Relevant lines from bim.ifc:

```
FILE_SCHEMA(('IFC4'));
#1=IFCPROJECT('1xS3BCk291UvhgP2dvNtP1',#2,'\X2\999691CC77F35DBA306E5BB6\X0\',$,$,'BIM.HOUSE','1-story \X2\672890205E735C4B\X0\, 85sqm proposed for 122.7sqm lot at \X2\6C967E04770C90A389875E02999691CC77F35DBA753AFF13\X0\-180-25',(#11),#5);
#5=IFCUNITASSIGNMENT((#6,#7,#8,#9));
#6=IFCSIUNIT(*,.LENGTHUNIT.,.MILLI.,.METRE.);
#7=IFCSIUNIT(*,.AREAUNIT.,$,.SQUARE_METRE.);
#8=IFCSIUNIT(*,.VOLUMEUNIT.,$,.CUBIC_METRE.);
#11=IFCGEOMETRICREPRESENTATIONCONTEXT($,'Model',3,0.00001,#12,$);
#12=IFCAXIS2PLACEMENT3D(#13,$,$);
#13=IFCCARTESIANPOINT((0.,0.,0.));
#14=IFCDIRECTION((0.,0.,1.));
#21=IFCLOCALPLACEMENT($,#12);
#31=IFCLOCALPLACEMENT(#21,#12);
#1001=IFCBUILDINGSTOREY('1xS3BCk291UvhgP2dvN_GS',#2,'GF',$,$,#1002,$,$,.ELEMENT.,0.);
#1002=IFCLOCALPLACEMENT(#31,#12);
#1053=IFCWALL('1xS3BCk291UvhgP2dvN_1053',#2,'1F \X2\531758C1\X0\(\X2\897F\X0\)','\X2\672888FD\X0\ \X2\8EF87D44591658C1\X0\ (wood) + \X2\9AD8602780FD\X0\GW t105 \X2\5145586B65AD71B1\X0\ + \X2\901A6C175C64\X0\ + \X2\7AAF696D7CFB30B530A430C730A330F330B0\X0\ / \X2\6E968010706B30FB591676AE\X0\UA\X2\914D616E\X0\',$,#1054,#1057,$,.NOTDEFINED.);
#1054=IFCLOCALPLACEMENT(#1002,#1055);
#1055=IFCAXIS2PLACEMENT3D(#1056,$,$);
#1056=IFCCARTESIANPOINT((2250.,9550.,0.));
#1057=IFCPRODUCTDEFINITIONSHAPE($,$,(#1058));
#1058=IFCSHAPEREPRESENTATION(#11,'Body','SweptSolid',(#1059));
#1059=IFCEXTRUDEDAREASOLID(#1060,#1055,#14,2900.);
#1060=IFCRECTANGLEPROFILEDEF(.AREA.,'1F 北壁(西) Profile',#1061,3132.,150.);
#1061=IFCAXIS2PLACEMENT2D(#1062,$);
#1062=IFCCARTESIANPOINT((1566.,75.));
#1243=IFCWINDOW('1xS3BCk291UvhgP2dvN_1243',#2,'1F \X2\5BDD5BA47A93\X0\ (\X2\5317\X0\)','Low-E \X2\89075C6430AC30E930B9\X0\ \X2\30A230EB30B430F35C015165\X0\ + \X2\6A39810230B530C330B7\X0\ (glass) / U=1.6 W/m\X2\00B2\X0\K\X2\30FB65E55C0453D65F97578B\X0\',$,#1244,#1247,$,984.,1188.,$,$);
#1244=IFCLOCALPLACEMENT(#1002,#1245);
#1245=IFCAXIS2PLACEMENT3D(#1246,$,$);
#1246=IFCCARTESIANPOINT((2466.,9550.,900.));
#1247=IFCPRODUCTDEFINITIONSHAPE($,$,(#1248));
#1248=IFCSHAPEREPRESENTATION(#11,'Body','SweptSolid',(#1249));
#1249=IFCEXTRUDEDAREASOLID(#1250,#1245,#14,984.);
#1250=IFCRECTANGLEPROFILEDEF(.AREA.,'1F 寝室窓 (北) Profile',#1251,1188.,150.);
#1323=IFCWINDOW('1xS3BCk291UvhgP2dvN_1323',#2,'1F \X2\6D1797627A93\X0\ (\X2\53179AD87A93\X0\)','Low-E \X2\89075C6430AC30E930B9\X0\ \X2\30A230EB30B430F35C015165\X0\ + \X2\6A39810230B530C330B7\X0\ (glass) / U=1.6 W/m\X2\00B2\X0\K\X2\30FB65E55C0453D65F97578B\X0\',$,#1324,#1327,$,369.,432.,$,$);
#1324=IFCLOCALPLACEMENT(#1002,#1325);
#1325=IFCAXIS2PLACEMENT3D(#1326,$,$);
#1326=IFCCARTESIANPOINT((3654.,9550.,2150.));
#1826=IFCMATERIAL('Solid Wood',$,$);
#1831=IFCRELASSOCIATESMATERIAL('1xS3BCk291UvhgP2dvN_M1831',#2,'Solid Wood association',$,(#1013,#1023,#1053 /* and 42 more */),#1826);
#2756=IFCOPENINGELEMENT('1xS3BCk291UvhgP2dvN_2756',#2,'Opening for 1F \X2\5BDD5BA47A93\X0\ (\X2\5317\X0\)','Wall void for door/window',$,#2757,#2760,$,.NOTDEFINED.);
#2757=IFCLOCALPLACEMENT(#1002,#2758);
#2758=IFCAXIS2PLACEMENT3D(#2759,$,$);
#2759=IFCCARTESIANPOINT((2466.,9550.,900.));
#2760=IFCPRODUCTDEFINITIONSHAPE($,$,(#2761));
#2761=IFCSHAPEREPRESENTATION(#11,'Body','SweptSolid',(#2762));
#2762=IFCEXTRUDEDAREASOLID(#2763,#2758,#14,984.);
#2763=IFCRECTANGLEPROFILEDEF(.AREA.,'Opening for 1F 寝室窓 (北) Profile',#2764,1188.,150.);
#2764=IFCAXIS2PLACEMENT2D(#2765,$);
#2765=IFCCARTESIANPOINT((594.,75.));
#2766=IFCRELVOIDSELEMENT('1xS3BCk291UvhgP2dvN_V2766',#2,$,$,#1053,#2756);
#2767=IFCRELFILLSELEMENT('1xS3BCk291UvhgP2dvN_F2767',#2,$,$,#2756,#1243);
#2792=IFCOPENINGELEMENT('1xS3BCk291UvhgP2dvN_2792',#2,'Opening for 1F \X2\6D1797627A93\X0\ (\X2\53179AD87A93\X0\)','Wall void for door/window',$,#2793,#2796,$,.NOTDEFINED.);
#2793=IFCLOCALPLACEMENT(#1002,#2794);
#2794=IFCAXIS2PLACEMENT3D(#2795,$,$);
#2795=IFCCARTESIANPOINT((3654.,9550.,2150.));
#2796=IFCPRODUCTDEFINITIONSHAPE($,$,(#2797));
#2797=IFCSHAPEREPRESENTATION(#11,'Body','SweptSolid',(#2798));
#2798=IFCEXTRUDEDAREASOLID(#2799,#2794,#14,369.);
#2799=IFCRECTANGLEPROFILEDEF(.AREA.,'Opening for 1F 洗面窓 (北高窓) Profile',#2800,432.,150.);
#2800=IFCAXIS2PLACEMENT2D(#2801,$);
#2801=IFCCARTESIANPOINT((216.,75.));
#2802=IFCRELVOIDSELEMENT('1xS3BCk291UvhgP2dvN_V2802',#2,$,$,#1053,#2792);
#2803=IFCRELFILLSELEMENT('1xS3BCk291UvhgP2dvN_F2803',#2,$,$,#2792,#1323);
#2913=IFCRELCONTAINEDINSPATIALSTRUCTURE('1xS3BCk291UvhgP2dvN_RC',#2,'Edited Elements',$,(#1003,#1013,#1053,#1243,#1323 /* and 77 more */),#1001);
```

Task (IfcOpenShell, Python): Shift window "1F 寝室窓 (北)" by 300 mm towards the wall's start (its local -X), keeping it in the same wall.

```python
import ifcopenshell
import ifcopenshell.api.geometry
import ifcopenshell.util.placement

model = ifcopenshell.open("bim.ifc")

window = model.by_guid("1xS3BCk291UvhgP2dvN_1243")
opening = window.FillsVoids[0].RelatingOpeningElement
wall = opening.VoidsElements[0].RelatingBuildingElement

wall_matrix = ifcopenshell.util.placement.get_local_placement(wall.ObjectPlacement)
shift = wall_matrix[:3, 0] * -300.0
before = ifcopenshell.util.placement.get_local_placement(window.ObjectPlacement)[:3, 3].copy()

# The window is not placed relative to its opening, so move both.
for product in (opening, window):
    matrix = ifcopenshell.util.placement.get_local_placement(product.ObjectPlacement)
    matrix[:3, 3] += shift
    ifcopenshell.api.geometry.edit_object_placement(model, product=product, matrix=matrix, is_si=False)

after = ifcopenshell.util.placement.get_local_placement(window.ObjectPlacement)[:3, 3]
print("window moved by", (after - before).round(3) + 0.0)

model.write("bim-out.ifc")
```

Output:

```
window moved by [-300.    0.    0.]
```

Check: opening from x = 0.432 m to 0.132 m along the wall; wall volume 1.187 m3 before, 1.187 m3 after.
